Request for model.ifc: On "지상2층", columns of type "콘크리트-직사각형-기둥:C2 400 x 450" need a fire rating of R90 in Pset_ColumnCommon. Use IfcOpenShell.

First a look at what the model holds.

```python
import ifcopenshell
import ifcopenshell.util.element

model = ifcopenshell.open("model.ifc")
print(model.schema)
storey = next(s for s in model.by_type("IfcBuildingStorey") if s.Name == "지상2층")
columns = [e for e in ifcopenshell.util.element.get_decomposition(storey) if e.is_a("IfcColumn")]
seen = {}
for e in columns:
    element_type = ifcopenshell.util.element.get_type(e)
    key = (element_type.Name if element_type != e and element_type else None, ifcopenshell.util.element.get_pset(e, "Pset_ColumnCommon", "FireRating"))
    seen[key] = seen.get(key, 0) + 1
for (name, value), count in sorted(seen.items(), key=str):
    print(count, "x", name, "|", value)
```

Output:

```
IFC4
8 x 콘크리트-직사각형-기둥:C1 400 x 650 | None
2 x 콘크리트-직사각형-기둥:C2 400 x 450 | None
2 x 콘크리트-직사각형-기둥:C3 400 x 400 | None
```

```python
import ifcopenshell
import ifcopenshell.api.pset
import ifcopenshell.util.element

model = ifcopenshell.open("model.ifc")

storey = next(s for s in model.by_type("IfcBuildingStorey") if s.Name == "지상2층")
columns = [e for e in ifcopenshell.util.element.get_decomposition(storey) if e.is_a("IfcColumn")]

count = 0
for e in columns:
    element_type = ifcopenshell.util.element.get_type(e)
    if element_type in (None, e) or element_type.Name != "콘크리트-직사각형-기둥:C2 400 x 450":
        continue
    # add_pset returns the element's existing set when there is one.
    pset = ifcopenshell.api.pset.add_pset(model, product=e, name="Pset_ColumnCommon")
    ifcopenshell.api.pset.edit_pset(model, pset=pset, properties={"FireRating": "R90"})
    count += 1

print(count, "columns updated")

model.write("model_updated.ifc")
```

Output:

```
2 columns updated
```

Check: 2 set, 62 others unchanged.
